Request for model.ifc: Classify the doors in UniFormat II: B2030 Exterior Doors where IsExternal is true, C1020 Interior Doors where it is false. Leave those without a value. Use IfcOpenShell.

First a look at what the model holds.

```python
import ifcopenshell
import ifcopenshell.util.element

model = ifcopenshell.open("model.ifc")
print(model.schema)
print("classifications:", [c.Name for c in model.by_type("IfcClassification")])
values = [ifcopenshell.util.element.get_pset(e, "Pset_DoorCommon", "IsExternal") for e in model.by_type("IfcDoor")]
for value in (True, False, None):
    print("IsExternal", value, values.count(value))
```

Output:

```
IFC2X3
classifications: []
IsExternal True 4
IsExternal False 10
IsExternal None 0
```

```python
import ifcopenshell
import ifcopenshell.api.classification
import ifcopenshell.util.element

model = ifcopenshell.open("model.ifc")

# IFC2X3 requires Source and Edition and has no link from the project to the system.
system = model.create_entity("IfcClassification", Source="ASTM", Edition="E1557", Name="UniFormat II")

doors = model.by_type("IfcDoor")
external = {e: ifcopenshell.util.element.get_pset(e, "Pset_DoorCommon", "IsExternal") for e in doors}
for flag, code, name in ((True, "B2030", "Exterior Doors"), (False, "C1020", "Interior Doors")):
    products = [e for e in doors if external[e] is flag]
    ifcopenshell.api.classification.add_reference(
        model, products=products, classification=system, identification=code, name=name
    )
    print(code, len(products))

model.write("model_edited.ifc")
```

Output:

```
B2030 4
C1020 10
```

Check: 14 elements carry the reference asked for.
